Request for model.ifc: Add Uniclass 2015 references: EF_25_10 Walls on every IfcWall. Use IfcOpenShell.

First a look at what the model holds.

```python
import ifcopenshell

model = ifcopenshell.open("model.ifc")
print(model.schema)
print("classifications:", [c.Name for c in model.by_type("IfcClassification")])
for ifc_class in ("IfcDoor", "IfcRoof", "IfcStair", "IfcWall", "IfcWindow"):
    print(ifc_class, len(model.by_type(ifc_class)))
```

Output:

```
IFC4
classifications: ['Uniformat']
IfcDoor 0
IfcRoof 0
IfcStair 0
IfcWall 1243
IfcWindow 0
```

```python
import ifcopenshell
import ifcopenshell.api.classification

model = ifcopenshell.open("model.ifc")

system = ifcopenshell.api.classification.add_classification(model, classification="Uniclass 2015")

codes = {
    "IfcWall": ("EF_25_10", "Walls"),
}
for ifc_class, (code, name) in codes.items():
    products = model.by_type(ifc_class)
    ifcopenshell.api.classification.add_reference(
        model, products=products, classification=system, identification=code, name=name
    )
    print(code, len(products))

model.write("model-out.ifc")
```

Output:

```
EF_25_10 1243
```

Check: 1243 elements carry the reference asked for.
